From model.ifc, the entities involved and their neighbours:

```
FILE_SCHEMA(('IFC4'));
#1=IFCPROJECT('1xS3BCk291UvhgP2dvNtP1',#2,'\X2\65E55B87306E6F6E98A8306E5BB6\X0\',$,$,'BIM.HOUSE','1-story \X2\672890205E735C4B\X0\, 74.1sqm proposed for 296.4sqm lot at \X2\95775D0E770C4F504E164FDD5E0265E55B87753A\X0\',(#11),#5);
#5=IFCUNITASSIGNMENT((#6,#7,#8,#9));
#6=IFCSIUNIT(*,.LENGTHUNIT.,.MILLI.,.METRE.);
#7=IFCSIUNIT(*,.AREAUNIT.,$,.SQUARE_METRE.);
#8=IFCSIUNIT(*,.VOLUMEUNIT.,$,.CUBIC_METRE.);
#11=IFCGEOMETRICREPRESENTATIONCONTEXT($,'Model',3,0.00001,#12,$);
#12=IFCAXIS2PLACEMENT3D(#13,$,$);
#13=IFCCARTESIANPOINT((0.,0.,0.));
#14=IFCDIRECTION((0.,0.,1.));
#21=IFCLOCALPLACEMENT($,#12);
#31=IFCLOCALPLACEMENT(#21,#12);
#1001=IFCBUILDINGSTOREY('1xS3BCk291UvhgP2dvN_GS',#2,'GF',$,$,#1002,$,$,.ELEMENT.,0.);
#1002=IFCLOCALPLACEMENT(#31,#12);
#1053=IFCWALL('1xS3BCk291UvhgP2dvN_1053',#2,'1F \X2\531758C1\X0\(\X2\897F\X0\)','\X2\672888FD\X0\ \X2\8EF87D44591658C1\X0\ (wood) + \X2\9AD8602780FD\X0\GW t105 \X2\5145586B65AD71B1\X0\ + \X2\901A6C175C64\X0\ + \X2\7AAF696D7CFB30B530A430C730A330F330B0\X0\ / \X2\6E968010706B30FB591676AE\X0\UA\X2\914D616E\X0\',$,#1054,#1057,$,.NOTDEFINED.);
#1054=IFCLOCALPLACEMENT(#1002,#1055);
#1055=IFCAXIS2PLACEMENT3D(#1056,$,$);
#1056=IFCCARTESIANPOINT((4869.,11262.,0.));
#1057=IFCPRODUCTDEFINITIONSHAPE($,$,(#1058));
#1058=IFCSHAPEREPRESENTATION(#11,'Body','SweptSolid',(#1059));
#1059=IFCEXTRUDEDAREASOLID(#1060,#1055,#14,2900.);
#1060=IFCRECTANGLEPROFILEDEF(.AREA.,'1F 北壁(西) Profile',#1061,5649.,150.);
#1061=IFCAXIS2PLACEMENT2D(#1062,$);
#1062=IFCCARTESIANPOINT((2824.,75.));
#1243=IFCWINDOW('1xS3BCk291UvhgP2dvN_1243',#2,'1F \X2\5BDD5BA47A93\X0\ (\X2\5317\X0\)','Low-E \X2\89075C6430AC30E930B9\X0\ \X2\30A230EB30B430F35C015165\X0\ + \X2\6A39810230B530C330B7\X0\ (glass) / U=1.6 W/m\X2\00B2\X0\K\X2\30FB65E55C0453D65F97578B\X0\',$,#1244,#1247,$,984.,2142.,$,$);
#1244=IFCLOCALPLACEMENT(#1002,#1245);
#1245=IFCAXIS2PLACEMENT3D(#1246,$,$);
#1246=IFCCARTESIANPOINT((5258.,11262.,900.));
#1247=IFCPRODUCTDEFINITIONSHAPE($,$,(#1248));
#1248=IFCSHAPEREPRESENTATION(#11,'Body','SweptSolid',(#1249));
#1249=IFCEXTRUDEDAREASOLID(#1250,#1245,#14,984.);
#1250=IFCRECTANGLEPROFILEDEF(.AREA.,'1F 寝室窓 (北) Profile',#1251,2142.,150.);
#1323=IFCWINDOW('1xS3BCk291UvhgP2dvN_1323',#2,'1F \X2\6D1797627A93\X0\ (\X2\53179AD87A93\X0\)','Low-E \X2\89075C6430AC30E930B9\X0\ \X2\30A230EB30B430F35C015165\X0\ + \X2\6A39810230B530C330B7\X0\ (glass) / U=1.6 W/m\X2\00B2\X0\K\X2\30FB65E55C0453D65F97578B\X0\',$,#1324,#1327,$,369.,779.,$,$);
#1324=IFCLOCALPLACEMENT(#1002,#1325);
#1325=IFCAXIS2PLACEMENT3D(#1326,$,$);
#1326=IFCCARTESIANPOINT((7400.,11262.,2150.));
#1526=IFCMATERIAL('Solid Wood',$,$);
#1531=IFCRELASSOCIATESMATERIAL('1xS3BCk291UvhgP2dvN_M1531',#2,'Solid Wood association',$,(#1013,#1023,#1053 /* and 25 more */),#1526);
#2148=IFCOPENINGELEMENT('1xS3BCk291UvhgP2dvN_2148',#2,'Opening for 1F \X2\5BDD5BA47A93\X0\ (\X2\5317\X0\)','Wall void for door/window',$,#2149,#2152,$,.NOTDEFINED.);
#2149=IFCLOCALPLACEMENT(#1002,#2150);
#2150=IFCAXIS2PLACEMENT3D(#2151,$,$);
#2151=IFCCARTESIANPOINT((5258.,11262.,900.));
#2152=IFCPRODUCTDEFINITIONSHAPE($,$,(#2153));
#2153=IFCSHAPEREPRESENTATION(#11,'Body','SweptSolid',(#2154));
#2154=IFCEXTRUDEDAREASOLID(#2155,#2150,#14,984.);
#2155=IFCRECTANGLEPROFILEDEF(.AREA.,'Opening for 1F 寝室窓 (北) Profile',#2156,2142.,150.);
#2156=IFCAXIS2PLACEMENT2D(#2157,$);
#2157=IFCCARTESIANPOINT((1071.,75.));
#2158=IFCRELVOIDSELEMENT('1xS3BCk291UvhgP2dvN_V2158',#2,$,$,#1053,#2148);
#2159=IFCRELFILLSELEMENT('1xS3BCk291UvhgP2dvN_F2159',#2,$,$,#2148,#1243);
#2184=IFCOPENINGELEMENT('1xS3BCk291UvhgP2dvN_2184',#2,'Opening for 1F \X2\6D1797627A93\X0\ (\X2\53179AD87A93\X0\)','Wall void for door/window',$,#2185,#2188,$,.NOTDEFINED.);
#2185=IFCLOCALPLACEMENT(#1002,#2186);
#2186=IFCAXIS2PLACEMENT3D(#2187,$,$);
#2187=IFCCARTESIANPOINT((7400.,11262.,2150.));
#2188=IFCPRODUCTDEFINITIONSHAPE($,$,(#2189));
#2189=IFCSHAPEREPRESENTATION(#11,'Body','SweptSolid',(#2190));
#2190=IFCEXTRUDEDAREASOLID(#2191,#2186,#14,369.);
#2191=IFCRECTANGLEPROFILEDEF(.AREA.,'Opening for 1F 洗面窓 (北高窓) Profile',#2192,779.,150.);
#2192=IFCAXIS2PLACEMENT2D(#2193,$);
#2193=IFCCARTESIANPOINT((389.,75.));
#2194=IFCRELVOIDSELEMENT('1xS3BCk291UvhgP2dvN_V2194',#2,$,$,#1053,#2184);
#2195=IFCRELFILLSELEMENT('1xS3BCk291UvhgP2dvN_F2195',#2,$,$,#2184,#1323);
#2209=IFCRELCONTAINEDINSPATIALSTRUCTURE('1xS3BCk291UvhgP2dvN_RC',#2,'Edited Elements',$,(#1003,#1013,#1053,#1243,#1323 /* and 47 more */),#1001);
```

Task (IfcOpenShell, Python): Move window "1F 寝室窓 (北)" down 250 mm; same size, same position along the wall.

```python
import numpy as np
import ifcopenshell
import ifcopenshell.api.geometry
import ifcopenshell.util.placement
import ifcopenshell.util.unit

model = ifcopenshell.open("model.ifc")
unit_scale = ifcopenshell.util.unit.calculate_unit_scale(model)

window = model.by_guid("1xS3BCk291UvhgP2dvN_1243")
opening = window.FillsVoids[0].RelatingOpeningElement
dz = -0.25 / unit_scale

shift = np.array([0.0, 0.0, dz])
# The window is not placed relative to its opening, so move both.
for product in (opening, window):
    matrix = ifcopenshell.util.placement.get_local_placement(product.ObjectPlacement)
    matrix[:3, 3] += shift
    ifcopenshell.api.geometry.edit_object_placement(model, product=product, matrix=matrix, is_si=False)

print(f"moved by {dz * unit_scale:+.3f} m")

model.write("model_edited.ifc")
```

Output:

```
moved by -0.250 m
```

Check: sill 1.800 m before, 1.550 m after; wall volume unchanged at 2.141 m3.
